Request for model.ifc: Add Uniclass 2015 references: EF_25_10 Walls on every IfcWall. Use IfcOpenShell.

First a look at what the model holds.

```python
import ifcopenshell

model = ifcopenshell.open("model.ifc")
print(model.schema)
print("classifications:", [c.Name for c in model.by_type("IfcClassification")])
for ifc_class in ("IfcDoor", "IfcRoof", "IfcStair", "IfcWall", "IfcWindow"):
    print(ifc_class, len(model.by_type(ifc_class)))
```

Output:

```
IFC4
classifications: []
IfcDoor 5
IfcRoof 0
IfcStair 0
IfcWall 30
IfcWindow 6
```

```python
import ifcopenshell
import ifcopenshell.api.classification

model = ifcopenshell.open("model.ifc")

system = ifcopenshell.api.classification.add_classification(model, classification="Uniclass 2015")

codes = {
    "IfcWall": ("EF_25_10", "Walls"),
}
for ifc_class, (code, name) in codes.items():
    products = model.by_type(ifc_class)
    ifcopenshell.api.classification.add_reference(
        model, products=products, classification=system, identification=code, name=name
    )
    print(code, len(products))

model.write("model_v2.ifc")
```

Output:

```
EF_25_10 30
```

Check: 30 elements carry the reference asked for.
